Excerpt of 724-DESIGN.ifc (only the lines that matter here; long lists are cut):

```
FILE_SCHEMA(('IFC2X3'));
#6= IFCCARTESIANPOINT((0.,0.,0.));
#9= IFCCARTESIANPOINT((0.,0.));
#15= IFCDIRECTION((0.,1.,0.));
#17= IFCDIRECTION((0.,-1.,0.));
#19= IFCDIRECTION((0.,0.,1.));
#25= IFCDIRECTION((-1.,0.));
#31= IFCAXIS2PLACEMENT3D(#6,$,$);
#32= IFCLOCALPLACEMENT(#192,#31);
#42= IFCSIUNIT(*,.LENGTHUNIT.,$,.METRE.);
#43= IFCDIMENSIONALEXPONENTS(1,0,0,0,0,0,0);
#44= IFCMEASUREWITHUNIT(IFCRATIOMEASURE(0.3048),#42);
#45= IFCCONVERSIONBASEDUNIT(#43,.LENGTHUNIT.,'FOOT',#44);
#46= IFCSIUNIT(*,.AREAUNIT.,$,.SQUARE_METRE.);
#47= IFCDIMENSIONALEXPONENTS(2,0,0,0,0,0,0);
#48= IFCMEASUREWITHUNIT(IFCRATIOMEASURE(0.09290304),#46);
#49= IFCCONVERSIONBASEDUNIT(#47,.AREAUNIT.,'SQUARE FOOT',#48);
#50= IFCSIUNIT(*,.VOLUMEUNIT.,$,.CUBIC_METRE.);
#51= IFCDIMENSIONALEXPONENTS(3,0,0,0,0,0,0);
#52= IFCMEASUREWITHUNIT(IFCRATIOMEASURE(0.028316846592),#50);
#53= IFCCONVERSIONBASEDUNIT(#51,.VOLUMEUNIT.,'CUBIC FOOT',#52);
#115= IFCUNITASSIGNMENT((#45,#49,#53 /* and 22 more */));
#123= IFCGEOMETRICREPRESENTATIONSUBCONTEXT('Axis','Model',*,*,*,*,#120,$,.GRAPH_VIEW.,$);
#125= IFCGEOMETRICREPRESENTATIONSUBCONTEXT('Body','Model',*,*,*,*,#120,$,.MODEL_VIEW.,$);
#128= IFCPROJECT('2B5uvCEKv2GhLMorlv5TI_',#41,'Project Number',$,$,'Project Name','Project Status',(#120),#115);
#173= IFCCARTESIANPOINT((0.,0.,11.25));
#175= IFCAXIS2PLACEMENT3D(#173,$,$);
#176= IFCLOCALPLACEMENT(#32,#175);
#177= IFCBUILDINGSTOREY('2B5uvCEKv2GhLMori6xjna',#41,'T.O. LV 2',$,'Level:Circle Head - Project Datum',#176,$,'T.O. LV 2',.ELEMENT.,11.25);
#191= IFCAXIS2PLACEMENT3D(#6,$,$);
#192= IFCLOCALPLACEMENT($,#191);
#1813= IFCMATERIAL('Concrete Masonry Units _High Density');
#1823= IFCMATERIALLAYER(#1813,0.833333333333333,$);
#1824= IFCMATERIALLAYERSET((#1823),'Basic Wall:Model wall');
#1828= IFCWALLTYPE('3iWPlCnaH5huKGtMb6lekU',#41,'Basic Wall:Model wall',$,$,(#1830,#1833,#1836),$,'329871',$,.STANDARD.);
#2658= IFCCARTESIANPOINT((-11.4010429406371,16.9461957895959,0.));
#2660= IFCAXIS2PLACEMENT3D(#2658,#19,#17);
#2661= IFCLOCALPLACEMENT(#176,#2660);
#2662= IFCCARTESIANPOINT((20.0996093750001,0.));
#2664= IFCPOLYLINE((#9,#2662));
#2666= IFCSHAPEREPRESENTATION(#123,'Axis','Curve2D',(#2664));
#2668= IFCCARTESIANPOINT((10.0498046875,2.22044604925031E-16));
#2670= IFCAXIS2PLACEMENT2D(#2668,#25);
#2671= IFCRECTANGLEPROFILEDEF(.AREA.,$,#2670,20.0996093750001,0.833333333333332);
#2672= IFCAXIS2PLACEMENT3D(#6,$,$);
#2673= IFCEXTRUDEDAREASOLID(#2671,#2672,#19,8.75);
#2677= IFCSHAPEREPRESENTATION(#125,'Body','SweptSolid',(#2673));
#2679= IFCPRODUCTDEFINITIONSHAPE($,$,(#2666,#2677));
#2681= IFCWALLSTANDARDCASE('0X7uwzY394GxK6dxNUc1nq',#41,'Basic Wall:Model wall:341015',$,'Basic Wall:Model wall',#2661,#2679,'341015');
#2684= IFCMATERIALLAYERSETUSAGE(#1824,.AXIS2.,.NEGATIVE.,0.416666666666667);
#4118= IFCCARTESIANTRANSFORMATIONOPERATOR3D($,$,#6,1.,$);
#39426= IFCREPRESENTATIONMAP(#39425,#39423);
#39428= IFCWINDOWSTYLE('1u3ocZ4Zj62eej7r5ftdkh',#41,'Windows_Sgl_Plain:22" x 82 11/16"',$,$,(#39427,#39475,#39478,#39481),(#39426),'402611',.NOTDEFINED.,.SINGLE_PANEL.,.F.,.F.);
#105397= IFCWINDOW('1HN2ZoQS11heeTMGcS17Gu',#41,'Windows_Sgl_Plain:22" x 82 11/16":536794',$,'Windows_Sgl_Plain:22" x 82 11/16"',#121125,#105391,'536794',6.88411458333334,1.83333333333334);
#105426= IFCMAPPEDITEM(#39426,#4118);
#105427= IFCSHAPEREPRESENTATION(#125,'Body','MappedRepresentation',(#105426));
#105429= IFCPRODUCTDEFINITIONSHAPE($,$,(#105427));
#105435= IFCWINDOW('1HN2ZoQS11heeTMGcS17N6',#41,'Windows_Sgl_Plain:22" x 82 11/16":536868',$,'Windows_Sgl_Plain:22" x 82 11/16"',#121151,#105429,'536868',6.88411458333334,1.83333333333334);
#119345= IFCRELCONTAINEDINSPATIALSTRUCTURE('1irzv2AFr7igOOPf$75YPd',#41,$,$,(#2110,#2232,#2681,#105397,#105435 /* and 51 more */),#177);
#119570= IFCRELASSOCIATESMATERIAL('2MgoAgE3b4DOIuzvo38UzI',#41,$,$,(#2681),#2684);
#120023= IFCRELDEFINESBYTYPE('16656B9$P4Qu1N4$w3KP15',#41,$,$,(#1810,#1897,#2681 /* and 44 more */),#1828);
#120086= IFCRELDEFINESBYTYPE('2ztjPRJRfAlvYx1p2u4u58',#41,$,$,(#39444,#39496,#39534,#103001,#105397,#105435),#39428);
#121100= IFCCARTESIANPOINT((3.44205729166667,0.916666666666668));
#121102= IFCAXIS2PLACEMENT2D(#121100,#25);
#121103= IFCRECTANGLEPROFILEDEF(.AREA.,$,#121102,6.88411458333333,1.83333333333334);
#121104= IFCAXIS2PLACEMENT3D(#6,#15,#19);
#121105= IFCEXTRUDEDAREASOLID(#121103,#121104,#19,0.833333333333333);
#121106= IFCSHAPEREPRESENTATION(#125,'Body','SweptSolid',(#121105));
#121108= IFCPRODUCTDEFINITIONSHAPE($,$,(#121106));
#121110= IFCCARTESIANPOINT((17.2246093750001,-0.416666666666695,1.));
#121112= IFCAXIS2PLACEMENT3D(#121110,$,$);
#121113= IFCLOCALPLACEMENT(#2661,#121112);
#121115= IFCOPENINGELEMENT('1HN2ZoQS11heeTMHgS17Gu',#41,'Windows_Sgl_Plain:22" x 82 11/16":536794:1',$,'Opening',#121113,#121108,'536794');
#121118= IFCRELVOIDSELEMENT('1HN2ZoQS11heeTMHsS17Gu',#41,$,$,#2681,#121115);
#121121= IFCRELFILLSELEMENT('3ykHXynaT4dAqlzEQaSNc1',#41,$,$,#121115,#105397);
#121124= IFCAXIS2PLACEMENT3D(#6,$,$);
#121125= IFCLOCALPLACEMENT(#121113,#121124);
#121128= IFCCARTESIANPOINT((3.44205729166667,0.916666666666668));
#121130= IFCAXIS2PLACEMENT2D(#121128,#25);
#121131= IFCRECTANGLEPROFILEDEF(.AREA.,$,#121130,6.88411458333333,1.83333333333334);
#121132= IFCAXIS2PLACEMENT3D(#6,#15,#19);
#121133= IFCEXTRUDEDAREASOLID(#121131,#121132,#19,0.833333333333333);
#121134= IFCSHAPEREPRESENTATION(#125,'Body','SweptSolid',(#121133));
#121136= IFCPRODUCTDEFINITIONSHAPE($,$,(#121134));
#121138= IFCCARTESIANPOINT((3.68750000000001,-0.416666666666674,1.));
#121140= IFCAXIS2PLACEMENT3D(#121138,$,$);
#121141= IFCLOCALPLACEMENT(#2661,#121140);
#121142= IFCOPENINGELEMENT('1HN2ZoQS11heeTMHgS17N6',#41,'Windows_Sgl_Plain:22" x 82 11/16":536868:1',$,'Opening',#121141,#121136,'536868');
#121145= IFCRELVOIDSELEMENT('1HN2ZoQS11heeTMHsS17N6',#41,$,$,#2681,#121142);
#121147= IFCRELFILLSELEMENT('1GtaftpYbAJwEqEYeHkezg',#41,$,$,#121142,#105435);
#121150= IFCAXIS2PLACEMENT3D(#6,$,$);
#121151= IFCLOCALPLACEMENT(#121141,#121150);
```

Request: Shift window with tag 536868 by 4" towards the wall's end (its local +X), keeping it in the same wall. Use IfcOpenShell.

```python
import ifcopenshell
import ifcopenshell.api.geometry
import ifcopenshell.util.placement
import ifcopenshell.util.unit

model = ifcopenshell.open("724-DESIGN.ifc")
unit_scale = ifcopenshell.util.unit.calculate_unit_scale(model)

window = model.by_guid("1HN2ZoQS11heeTMGcS17N6")
opening = window.FillsVoids[0].RelatingOpeningElement
wall = opening.VoidsElements[0].RelatingBuildingElement

wall_matrix = ifcopenshell.util.placement.get_local_placement(wall.ObjectPlacement)
shift = wall_matrix[:3, 0] * 4 * 0.0254 / unit_scale
before = ifcopenshell.util.placement.get_local_placement(window.ObjectPlacement)[:3, 3].copy()

# The window is placed relative to its opening, so it follows when the opening moves.
matrix = ifcopenshell.util.placement.get_local_placement(opening.ObjectPlacement)
matrix[:3, 3] += shift
ifcopenshell.api.geometry.edit_object_placement(
    model, product=opening, matrix=matrix, is_si=False, should_transform_children=True
)

after = ifcopenshell.util.placement.get_local_placement(window.ObjectPlacement)[:3, 3]
print("window moved by", (after - before).round(3) + 0.0)

model.write("724-DESIGN_v2.ifc")
```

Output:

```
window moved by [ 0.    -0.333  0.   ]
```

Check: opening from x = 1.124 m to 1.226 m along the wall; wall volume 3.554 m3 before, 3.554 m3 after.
